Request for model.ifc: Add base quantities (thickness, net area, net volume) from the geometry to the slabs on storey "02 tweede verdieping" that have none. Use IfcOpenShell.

First a look at what the model holds.

```python
import ifcopenshell
import ifcopenshell.util.element
import ifcopenshell.util.unit

model = ifcopenshell.open("model.ifc")
print(model.schema)
for unit_type in ("LENGTHUNIT", "AREAUNIT", "VOLUMEUNIT"):
    print(unit_type, ifcopenshell.util.unit.calculate_unit_scale(model, unit_type))
storey = next(s for s in model.by_type("IfcBuildingStorey") if s.Name == "02 tweede verdieping")
slabs = [e for e in ifcopenshell.util.element.get_decomposition(storey) if e.is_a("IfcSlab")]
for e in sorted(slabs, key=lambda e: e.id()):
    print(e.id(), e.is_a(), e.Name, list(ifcopenshell.util.element.get_psets(e, qtos_only=True)), sep=" | ")
```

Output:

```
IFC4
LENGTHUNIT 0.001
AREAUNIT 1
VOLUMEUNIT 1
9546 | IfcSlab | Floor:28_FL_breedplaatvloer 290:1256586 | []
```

```python
import ifcopenshell
import ifcopenshell.api.pset
import ifcopenshell.geom
import ifcopenshell.util.element
import ifcopenshell.util.shape
import ifcopenshell.util.unit

model = ifcopenshell.open("model.ifc")
unit_scale = ifcopenshell.util.unit.calculate_unit_scale(model)
area_scale = ifcopenshell.util.unit.calculate_unit_scale(model, "AREAUNIT")
volume_scale = ifcopenshell.util.unit.calculate_unit_scale(model, "VOLUMEUNIT")
settings = ifcopenshell.geom.settings()

storey = next(s for s in model.by_type("IfcBuildingStorey") if s.Name == "02 tweede verdieping")
slabs = [e for e in ifcopenshell.util.element.get_decomposition(storey) if e.is_a("IfcSlab")]

for e in sorted(slabs, key=lambda e: e.id()):
    if ifcopenshell.util.element.get_psets(e, qtos_only=True, should_inherit=False):
        continue
    # Geometry comes back in metres, in the element's own axes.
    shape = ifcopenshell.geom.create_shape(settings, e)
    values = {
        "Width": ifcopenshell.util.shape.get_z(shape.geometry) / unit_scale,
        "NetArea": ifcopenshell.util.shape.get_footprint_area(shape.geometry) / area_scale,
        "NetVolume": ifcopenshell.util.shape.get_volume(shape.geometry) / volume_scale,
    }
    qto = ifcopenshell.api.pset.add_qto(model, product=e, name="Qto_SlabBaseQuantities")
    ifcopenshell.api.pset.edit_qto(model, qto=qto, properties=values)
    print(e.id(), {k: round(v, 3) for k, v in values.items()})

model.write("model_v2.ifc")
```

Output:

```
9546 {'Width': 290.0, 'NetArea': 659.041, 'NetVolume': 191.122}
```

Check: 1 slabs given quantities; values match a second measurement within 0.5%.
